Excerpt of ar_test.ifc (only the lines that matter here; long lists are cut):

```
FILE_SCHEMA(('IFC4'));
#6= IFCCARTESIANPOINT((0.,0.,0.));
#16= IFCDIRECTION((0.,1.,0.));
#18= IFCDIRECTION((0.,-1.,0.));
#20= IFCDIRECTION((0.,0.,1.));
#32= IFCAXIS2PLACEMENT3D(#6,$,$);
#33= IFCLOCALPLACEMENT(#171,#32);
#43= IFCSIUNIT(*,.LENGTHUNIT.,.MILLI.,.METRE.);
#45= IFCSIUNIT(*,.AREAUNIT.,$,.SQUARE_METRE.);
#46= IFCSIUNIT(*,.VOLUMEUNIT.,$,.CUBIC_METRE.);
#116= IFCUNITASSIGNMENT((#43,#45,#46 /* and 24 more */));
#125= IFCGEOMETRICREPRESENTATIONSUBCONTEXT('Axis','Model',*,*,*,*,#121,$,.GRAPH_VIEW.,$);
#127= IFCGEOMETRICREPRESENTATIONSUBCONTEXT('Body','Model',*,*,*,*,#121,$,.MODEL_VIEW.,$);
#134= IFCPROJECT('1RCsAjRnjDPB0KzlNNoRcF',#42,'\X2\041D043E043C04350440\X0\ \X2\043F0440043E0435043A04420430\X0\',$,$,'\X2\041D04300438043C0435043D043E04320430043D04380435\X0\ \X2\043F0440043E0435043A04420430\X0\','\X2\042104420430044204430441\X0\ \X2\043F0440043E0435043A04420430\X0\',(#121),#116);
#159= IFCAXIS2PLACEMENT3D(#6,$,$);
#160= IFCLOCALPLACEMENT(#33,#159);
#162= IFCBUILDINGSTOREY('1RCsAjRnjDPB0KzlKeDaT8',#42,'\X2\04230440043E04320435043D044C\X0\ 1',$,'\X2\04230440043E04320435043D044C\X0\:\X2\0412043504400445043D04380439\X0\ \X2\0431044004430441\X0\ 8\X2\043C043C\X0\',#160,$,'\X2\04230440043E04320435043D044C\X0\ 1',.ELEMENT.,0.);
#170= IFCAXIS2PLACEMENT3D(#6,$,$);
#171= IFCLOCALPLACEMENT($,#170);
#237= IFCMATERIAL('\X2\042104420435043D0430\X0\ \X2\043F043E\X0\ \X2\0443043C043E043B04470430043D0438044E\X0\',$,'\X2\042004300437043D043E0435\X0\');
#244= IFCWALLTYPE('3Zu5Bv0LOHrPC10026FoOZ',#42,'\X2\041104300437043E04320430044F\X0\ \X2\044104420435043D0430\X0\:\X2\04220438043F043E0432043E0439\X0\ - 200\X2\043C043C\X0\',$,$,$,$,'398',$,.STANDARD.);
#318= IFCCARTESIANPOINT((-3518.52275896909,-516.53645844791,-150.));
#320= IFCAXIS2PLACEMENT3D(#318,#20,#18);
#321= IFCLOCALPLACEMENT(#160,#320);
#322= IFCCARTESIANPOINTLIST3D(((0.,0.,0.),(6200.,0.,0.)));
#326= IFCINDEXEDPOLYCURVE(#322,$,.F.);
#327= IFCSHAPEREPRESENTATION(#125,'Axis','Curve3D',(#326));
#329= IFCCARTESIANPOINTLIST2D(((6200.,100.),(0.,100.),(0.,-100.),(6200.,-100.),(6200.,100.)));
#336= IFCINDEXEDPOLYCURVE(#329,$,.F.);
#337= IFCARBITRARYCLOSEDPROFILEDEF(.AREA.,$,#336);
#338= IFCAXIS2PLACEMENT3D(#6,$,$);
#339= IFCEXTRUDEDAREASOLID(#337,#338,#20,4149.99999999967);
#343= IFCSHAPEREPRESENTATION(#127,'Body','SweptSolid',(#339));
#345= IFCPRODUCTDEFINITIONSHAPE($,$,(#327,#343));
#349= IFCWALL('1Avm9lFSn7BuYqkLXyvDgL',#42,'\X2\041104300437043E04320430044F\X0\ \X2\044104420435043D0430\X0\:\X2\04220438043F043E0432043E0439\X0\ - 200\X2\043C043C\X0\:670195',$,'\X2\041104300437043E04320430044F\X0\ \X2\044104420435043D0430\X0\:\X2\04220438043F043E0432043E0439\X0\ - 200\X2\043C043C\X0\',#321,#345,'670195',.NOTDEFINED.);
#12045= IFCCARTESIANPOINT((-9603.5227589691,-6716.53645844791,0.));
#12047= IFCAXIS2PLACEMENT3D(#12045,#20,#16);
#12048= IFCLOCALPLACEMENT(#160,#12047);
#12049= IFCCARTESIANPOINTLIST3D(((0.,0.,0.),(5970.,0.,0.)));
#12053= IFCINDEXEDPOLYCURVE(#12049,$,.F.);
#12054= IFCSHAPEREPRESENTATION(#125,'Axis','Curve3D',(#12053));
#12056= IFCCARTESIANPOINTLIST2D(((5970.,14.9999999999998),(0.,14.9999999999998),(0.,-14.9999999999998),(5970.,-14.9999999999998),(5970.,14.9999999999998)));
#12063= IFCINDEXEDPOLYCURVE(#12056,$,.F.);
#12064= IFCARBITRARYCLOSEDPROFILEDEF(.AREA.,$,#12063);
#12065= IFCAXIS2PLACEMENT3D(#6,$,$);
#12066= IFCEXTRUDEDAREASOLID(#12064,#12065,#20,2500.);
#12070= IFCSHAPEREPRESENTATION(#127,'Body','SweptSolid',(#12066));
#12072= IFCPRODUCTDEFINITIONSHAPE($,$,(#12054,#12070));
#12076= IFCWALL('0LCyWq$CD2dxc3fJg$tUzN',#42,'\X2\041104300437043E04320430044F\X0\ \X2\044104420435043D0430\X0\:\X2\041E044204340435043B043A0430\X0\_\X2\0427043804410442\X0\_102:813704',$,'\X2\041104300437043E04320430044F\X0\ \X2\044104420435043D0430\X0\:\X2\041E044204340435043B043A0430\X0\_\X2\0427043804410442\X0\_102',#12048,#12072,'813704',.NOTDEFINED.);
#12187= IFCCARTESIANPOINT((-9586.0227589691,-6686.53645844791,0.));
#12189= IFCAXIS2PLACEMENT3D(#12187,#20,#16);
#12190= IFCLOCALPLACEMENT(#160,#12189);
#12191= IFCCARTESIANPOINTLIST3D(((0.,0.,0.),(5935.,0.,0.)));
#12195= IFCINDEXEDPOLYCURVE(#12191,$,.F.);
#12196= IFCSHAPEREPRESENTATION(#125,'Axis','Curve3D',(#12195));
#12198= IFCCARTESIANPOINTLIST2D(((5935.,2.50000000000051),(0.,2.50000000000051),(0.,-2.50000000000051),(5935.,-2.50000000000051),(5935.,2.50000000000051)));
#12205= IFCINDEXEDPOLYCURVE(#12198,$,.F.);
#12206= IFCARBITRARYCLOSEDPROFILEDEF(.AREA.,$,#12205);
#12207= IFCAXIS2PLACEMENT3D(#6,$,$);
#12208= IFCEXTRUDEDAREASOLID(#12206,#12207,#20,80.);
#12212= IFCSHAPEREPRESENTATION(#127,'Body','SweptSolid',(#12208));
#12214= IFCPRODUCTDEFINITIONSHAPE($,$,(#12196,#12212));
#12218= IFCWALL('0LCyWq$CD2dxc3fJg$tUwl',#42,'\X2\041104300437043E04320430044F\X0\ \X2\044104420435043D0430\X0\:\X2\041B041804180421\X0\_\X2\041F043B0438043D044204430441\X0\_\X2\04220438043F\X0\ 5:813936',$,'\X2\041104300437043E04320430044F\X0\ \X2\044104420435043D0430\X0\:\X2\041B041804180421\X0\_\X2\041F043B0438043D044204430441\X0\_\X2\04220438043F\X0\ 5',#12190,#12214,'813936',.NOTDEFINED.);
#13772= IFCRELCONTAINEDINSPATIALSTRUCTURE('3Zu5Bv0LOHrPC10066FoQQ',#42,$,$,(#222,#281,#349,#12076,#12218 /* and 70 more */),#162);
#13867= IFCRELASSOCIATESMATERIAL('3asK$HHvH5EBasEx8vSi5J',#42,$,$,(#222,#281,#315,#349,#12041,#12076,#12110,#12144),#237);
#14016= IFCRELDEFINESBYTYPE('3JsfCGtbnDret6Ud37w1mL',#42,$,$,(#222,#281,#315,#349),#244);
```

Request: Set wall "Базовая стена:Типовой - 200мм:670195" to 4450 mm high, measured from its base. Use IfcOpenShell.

```python
import ifcopenshell
import ifcopenshell.geom
import ifcopenshell.util.representation
import ifcopenshell.util.shape
import ifcopenshell.util.unit

model = ifcopenshell.open("ar_test.ifc")
unit_scale = ifcopenshell.util.unit.calculate_unit_scale(model)
settings = ifcopenshell.geom.settings()


def volume(element):
    """Net volume in cubic metres, openings subtracted."""
    shape = ifcopenshell.geom.create_shape(settings, element)
    return ifcopenshell.util.shape.get_volume(shape.geometry)


wall = model.by_guid("1Avm9lFSn7BuYqkLXyvDgL")
before = volume(wall)

body = ifcopenshell.util.representation.get_representation(wall, "Model", "Body")
solid = body.Items[0]
old_height = solid.Depth
solid.Depth = 4.45 / unit_scale
after = volume(wall)

print(f"height {old_height:g} -> {solid.Depth:g}, volume {before:.3f} -> {after:.3f} m3")

model.write("ar_test_v2.ifc")
```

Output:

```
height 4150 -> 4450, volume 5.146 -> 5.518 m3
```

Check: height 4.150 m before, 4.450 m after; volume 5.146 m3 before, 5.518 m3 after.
